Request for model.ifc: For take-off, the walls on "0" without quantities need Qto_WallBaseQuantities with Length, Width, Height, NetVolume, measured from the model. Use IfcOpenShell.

First a look at what the model holds.

```python
import ifcopenshell
import ifcopenshell.util.element
import ifcopenshell.util.unit

model = ifcopenshell.open("model.ifc")
print(model.schema)
for unit_type in ("LENGTHUNIT", "AREAUNIT", "VOLUMEUNIT"):
    print(unit_type, ifcopenshell.util.unit.calculate_unit_scale(model, unit_type))
storey = next(s for s in model.by_type("IfcBuildingStorey") if s.Name == "0")
walls = [e for e in ifcopenshell.util.element.get_decomposition(storey) if e.is_a("IfcWall")]
for e in sorted(walls, key=lambda e: e.id()):
    print(e.id(), e.is_a(), e.Name, list(ifcopenshell.util.element.get_psets(e, qtos_only=True)), sep=" | ")
```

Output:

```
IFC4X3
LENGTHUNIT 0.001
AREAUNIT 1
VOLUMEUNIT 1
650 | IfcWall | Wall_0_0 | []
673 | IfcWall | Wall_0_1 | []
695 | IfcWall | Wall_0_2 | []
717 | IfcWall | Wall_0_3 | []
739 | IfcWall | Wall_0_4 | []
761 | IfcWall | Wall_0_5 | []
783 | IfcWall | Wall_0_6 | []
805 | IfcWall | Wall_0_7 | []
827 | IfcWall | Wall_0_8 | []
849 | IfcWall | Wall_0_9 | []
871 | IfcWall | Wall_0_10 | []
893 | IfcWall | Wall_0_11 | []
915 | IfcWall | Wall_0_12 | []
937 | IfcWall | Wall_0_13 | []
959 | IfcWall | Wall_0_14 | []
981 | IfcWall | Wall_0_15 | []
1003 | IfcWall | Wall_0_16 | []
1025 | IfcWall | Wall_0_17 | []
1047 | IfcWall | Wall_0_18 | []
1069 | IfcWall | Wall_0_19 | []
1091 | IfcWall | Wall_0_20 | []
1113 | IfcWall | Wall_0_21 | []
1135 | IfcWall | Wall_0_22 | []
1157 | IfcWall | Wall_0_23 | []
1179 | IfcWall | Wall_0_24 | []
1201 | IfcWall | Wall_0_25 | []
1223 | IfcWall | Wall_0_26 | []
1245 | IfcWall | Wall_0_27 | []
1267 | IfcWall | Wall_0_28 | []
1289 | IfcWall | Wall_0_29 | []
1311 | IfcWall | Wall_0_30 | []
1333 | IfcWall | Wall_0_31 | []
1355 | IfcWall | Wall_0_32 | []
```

```python
import ifcopenshell
import ifcopenshell.api.pset
import ifcopenshell.geom
import ifcopenshell.util.element
import ifcopenshell.util.shape
import ifcopenshell.util.unit

model = ifcopenshell.open("model.ifc")
unit_scale = ifcopenshell.util.unit.calculate_unit_scale(model)
volume_scale = ifcopenshell.util.unit.calculate_unit_scale(model, "VOLUMEUNIT")
settings = ifcopenshell.geom.settings()

storey = next(s for s in model.by_type("IfcBuildingStorey") if s.Name == "0")
walls = [e for e in ifcopenshell.util.element.get_decomposition(storey) if e.is_a("IfcWall")]

for e in sorted(walls, key=lambda e: e.id()):
    if ifcopenshell.util.element.get_psets(e, qtos_only=True, should_inherit=False):
        continue
    # Geometry comes back in metres, in the element's own axes.
    shape = ifcopenshell.geom.create_shape(settings, e)
    values = {
        "Length": ifcopenshell.util.shape.get_x(shape.geometry) / unit_scale,
        "Width": ifcopenshell.util.shape.get_y(shape.geometry) / unit_scale,
        "Height": ifcopenshell.util.shape.get_z(shape.geometry) / unit_scale,
        "NetVolume": ifcopenshell.util.shape.get_volume(shape.geometry) / volume_scale,
    }
    qto = ifcopenshell.api.pset.add_qto(model, product=e, name="Qto_WallBaseQuantities")
    ifcopenshell.api.pset.edit_qto(model, qto=qto, properties=values)
    print(e.id(), {k: round(v, 3) for k, v in values.items()})

model.write("model_updated.ifc")
```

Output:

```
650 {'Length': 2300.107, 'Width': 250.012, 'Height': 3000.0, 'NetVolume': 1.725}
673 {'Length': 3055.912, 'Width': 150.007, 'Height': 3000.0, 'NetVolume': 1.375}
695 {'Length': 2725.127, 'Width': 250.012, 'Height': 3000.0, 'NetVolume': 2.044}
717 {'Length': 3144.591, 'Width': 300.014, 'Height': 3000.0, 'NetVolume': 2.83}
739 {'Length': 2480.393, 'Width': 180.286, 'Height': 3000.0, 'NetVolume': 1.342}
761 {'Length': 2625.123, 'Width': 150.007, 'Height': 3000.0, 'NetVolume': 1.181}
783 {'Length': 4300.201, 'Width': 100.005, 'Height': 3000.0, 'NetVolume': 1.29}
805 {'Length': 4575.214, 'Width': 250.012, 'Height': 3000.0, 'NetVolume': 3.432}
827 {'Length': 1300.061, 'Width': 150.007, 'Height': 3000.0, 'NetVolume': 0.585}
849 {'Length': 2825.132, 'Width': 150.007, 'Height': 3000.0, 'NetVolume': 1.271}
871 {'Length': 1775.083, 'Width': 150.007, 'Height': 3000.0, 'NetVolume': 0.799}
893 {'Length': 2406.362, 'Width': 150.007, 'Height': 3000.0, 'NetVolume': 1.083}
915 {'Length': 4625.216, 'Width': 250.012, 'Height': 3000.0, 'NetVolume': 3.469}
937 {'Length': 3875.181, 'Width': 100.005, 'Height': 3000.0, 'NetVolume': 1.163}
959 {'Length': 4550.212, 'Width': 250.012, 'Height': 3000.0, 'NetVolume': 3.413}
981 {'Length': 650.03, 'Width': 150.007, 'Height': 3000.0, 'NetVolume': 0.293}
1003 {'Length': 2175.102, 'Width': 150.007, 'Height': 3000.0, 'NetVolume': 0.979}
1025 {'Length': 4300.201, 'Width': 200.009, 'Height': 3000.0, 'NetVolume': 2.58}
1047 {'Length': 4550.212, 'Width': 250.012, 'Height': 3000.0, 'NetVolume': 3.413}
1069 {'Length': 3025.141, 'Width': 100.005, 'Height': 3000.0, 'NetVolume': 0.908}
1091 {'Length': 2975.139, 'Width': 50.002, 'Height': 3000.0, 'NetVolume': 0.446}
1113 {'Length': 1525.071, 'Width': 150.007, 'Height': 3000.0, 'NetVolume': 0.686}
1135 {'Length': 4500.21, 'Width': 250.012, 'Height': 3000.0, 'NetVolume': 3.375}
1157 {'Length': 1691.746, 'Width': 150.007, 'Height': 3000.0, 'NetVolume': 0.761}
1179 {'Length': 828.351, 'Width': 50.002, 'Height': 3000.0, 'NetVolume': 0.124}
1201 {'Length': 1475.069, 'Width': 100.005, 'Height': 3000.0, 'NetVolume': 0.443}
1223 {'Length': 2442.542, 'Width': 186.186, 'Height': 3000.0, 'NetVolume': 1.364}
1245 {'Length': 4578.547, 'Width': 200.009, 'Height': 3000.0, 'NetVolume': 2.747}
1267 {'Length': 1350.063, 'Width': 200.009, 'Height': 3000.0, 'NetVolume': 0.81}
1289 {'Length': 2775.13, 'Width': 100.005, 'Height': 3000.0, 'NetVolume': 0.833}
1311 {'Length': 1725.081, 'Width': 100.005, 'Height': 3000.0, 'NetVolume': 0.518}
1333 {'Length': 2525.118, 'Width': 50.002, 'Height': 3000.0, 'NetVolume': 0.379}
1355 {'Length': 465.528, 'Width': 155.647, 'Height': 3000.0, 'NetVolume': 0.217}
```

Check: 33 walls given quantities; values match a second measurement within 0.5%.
